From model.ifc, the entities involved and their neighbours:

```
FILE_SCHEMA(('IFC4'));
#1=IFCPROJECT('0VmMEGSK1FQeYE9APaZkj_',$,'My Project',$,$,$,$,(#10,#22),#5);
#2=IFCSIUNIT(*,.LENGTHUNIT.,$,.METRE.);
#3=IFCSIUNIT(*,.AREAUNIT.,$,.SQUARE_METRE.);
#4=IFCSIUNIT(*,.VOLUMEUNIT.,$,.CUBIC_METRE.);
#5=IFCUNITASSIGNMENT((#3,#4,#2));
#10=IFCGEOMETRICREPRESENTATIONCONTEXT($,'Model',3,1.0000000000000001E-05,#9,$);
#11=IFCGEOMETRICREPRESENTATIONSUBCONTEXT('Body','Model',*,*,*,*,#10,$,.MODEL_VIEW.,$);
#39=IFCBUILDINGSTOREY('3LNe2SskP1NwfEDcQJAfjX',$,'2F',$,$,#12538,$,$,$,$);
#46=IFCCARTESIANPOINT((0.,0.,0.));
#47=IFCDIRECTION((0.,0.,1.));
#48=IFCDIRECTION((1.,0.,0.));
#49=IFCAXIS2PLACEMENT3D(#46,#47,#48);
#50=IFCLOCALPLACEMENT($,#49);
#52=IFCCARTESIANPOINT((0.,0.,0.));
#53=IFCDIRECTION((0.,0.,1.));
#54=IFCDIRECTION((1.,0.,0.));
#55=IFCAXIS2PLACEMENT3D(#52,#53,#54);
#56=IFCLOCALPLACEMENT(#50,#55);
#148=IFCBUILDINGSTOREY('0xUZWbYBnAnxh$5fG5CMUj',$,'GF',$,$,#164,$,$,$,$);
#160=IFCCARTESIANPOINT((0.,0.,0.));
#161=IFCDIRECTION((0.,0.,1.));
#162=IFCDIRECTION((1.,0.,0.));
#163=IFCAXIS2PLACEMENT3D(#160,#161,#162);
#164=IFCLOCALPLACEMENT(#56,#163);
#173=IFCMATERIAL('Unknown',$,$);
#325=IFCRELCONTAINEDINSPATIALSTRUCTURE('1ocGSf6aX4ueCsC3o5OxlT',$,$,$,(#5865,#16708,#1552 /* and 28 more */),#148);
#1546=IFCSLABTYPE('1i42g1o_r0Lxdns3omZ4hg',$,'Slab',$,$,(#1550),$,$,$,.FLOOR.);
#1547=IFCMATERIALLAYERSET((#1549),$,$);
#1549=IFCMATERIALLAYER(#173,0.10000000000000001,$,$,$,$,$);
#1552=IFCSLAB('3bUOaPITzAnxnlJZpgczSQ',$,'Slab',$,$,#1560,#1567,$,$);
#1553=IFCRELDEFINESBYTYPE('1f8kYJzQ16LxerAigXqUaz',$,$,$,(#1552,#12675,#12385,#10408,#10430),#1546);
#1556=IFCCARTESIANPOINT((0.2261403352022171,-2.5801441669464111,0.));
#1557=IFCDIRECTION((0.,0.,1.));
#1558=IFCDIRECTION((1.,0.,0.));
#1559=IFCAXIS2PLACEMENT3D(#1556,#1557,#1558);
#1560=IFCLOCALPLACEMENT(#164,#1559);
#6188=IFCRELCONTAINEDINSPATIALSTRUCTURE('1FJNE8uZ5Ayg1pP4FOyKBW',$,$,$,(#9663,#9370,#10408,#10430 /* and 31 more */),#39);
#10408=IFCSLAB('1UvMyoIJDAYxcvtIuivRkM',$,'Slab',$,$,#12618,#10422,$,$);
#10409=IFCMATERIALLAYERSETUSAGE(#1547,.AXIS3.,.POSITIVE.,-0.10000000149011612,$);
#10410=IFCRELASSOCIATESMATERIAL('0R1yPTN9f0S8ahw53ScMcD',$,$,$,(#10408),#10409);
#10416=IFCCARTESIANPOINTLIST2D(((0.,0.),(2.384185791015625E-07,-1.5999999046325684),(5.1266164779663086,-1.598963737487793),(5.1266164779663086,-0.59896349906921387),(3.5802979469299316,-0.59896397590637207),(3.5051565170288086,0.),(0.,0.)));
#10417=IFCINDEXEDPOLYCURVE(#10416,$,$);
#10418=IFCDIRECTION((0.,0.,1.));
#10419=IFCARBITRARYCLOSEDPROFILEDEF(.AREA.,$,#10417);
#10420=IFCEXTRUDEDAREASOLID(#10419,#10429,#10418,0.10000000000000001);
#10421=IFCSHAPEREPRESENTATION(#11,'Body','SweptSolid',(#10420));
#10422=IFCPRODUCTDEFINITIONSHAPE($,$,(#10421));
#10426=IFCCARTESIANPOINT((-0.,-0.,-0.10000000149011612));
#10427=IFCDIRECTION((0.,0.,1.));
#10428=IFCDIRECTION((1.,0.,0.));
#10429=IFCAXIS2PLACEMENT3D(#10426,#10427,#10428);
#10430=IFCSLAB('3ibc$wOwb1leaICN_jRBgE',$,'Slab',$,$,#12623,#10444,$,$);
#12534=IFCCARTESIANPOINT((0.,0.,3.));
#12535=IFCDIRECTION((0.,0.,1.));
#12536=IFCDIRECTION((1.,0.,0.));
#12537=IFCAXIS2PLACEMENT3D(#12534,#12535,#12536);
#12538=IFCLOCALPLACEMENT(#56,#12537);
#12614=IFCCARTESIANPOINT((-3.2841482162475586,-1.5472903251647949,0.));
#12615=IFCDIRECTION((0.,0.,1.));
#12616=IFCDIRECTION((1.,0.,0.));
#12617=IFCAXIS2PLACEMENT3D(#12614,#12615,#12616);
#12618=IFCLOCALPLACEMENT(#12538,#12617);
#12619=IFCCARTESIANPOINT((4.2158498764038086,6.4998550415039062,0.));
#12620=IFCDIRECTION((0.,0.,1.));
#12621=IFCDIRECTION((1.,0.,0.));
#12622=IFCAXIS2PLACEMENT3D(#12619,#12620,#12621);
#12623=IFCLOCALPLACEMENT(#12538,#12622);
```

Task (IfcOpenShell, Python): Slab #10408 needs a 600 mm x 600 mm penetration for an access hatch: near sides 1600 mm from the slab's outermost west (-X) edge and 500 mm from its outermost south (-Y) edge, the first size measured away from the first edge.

```python
import numpy as np
import ifcopenshell
import ifcopenshell.api.feature
import ifcopenshell.api.geometry
import ifcopenshell.api.root
import ifcopenshell.geom
import ifcopenshell.util.placement
import ifcopenshell.util.representation
import ifcopenshell.util.shape
import ifcopenshell.util.unit

model = ifcopenshell.open("model.ifc")
unit_scale = ifcopenshell.util.unit.calculate_unit_scale(model)
settings = ifcopenshell.geom.settings()


def volume(element):
    """Net volume in cubic metres, openings subtracted."""
    shape = ifcopenshell.geom.create_shape(settings, element)
    return ifcopenshell.util.shape.get_volume(shape.geometry)


slab = model.by_guid("1UvMyoIJDAYxcvtIuivRkM")
before = volume(slab)

# Extent in the slab's own axes, in metres. The edges named are its -X and -Y sides.
slab_shape = ifcopenshell.geom.create_shape(settings, slab)
vertices = ifcopenshell.util.shape.get_vertices(slab_shape.geometry)
x_min, y_min, bottom = vertices.min(axis=0)
top = vertices[:, 2].max()

opening = ifcopenshell.api.root.create_entity(model, ifc_class="IfcOpeningElement", name="Access hatch opening", predefined_type="OPENING")
context = ifcopenshell.util.representation.get_context(model, "Model", "Body", "MODEL_VIEW")
width, depth = 0.6, 0.6
outline = [(0.0, 0.0), (width, 0.0), (width, depth), (0.0, depth), (0.0, 0.0)]
# Overshoot both faces by 50 mm so the cut is clean.
shape = ifcopenshell.api.geometry.add_slab_representation(
    model, context=context, depth=top - bottom + 0.1, polyline=outline
)
ifcopenshell.api.geometry.assign_representation(model, product=opening, representation=shape)

matrix = ifcopenshell.util.placement.get_local_placement(slab.ObjectPlacement)
matrix[:, 3] = matrix @ np.append(np.array([x_min + 1.6, y_min + 0.5, bottom - 0.05]) / unit_scale, 1.0)
ifcopenshell.api.geometry.edit_object_placement(model, product=opening, matrix=matrix, is_si=False)
ifcopenshell.api.feature.add_feature(model, feature=opening, element=slab)

after = volume(slab)

print(f"slab volume {before:.3f} -> {after:.3f} m3")

model.write("model-out.ifc")
```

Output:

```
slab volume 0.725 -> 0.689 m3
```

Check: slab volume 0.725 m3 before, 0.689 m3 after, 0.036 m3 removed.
